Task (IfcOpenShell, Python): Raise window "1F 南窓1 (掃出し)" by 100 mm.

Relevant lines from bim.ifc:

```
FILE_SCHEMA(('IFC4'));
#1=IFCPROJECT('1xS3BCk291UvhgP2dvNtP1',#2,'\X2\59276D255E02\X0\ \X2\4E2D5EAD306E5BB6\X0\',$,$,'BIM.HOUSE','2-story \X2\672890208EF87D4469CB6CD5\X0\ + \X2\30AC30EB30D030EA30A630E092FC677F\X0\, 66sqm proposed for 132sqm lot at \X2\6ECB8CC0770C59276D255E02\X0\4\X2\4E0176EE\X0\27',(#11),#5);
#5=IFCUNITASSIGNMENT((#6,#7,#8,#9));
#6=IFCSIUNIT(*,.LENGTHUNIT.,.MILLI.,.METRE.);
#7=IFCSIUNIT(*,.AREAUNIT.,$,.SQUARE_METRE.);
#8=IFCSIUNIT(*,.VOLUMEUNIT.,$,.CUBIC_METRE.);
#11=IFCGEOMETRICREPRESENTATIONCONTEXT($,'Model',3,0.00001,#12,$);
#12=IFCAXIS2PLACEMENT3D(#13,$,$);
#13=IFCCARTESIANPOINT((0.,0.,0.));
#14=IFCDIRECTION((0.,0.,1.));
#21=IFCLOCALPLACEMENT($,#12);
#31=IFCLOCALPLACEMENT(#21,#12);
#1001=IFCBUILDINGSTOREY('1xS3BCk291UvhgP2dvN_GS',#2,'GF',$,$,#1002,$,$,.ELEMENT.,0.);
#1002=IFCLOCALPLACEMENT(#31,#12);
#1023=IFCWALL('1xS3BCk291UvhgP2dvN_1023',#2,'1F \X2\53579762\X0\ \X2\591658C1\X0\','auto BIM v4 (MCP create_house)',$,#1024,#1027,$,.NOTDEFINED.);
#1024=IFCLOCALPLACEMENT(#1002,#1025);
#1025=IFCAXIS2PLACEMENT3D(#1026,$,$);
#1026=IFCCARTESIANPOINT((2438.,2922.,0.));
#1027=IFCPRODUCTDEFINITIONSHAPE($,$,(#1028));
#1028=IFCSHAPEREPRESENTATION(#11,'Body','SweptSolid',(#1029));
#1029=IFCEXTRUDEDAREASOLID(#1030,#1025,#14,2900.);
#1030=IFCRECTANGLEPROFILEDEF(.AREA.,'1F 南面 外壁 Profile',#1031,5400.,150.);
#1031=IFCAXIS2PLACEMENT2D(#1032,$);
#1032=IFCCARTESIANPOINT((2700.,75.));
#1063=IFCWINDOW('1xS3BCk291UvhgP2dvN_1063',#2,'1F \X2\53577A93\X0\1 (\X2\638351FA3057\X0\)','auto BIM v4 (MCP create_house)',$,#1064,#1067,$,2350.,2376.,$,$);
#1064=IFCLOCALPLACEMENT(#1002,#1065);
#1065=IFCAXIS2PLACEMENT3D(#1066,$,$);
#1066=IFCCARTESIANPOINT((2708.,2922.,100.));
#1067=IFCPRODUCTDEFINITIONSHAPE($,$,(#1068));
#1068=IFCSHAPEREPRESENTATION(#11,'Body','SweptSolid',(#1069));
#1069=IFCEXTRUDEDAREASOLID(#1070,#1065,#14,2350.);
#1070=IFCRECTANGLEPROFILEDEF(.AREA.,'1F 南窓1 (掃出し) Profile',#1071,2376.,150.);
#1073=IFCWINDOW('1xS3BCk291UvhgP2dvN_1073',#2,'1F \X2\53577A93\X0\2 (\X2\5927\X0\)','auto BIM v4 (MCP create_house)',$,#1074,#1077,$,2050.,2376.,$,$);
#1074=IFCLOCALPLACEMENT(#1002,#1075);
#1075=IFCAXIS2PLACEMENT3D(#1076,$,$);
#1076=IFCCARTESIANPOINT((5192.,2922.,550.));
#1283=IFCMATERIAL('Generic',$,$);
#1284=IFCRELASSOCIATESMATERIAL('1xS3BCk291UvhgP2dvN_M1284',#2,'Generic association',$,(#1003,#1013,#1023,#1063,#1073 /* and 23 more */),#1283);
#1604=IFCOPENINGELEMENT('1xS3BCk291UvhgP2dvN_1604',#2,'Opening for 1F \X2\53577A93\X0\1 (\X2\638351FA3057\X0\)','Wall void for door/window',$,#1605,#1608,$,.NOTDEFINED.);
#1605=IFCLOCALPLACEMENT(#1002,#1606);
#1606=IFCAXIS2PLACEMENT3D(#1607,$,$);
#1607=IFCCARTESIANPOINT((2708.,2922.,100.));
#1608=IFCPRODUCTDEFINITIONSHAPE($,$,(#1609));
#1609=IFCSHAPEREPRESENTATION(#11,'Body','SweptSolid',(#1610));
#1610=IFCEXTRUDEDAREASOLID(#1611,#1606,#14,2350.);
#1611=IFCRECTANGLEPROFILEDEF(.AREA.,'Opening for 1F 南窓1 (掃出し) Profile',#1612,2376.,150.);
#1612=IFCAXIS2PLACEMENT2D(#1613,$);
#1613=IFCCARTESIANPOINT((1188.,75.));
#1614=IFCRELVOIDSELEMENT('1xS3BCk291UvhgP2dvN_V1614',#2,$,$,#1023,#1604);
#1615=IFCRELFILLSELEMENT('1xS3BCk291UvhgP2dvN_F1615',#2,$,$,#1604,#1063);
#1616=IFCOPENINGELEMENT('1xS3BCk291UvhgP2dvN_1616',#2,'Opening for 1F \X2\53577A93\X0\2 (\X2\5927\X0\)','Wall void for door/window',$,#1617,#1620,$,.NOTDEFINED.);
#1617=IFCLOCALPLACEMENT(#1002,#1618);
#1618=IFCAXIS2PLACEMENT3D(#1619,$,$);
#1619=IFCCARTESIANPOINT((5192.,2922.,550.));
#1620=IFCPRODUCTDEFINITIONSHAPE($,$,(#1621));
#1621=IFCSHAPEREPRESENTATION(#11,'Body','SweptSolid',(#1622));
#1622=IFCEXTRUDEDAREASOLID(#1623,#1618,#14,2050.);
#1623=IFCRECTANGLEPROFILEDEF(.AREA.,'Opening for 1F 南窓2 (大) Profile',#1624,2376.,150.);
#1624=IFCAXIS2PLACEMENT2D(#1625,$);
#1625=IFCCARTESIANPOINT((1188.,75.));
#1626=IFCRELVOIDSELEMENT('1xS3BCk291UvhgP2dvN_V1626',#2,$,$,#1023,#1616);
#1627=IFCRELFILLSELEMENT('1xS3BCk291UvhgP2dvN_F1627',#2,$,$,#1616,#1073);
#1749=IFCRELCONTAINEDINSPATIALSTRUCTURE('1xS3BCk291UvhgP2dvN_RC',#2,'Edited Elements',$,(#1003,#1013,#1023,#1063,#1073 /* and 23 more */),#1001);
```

```python
import numpy as np
import ifcopenshell
import ifcopenshell.api.geometry
import ifcopenshell.util.placement
import ifcopenshell.util.unit

model = ifcopenshell.open("bim.ifc")
unit_scale = ifcopenshell.util.unit.calculate_unit_scale(model)

window = model.by_guid("1xS3BCk291UvhgP2dvN_1063")
opening = window.FillsVoids[0].RelatingOpeningElement
dz = 0.1 / unit_scale

shift = np.array([0.0, 0.0, dz])
# The window is not placed relative to its opening, so move both.
for product in (opening, window):
    matrix = ifcopenshell.util.placement.get_local_placement(product.ObjectPlacement)
    matrix[:3, 3] += shift
    ifcopenshell.api.geometry.edit_object_placement(model, product=product, matrix=matrix, is_si=False)

print(f"moved by {dz * unit_scale:+.3f} m")

model.write("bim_edited.ifc")
```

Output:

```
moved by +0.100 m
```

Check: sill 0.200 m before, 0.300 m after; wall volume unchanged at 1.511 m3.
